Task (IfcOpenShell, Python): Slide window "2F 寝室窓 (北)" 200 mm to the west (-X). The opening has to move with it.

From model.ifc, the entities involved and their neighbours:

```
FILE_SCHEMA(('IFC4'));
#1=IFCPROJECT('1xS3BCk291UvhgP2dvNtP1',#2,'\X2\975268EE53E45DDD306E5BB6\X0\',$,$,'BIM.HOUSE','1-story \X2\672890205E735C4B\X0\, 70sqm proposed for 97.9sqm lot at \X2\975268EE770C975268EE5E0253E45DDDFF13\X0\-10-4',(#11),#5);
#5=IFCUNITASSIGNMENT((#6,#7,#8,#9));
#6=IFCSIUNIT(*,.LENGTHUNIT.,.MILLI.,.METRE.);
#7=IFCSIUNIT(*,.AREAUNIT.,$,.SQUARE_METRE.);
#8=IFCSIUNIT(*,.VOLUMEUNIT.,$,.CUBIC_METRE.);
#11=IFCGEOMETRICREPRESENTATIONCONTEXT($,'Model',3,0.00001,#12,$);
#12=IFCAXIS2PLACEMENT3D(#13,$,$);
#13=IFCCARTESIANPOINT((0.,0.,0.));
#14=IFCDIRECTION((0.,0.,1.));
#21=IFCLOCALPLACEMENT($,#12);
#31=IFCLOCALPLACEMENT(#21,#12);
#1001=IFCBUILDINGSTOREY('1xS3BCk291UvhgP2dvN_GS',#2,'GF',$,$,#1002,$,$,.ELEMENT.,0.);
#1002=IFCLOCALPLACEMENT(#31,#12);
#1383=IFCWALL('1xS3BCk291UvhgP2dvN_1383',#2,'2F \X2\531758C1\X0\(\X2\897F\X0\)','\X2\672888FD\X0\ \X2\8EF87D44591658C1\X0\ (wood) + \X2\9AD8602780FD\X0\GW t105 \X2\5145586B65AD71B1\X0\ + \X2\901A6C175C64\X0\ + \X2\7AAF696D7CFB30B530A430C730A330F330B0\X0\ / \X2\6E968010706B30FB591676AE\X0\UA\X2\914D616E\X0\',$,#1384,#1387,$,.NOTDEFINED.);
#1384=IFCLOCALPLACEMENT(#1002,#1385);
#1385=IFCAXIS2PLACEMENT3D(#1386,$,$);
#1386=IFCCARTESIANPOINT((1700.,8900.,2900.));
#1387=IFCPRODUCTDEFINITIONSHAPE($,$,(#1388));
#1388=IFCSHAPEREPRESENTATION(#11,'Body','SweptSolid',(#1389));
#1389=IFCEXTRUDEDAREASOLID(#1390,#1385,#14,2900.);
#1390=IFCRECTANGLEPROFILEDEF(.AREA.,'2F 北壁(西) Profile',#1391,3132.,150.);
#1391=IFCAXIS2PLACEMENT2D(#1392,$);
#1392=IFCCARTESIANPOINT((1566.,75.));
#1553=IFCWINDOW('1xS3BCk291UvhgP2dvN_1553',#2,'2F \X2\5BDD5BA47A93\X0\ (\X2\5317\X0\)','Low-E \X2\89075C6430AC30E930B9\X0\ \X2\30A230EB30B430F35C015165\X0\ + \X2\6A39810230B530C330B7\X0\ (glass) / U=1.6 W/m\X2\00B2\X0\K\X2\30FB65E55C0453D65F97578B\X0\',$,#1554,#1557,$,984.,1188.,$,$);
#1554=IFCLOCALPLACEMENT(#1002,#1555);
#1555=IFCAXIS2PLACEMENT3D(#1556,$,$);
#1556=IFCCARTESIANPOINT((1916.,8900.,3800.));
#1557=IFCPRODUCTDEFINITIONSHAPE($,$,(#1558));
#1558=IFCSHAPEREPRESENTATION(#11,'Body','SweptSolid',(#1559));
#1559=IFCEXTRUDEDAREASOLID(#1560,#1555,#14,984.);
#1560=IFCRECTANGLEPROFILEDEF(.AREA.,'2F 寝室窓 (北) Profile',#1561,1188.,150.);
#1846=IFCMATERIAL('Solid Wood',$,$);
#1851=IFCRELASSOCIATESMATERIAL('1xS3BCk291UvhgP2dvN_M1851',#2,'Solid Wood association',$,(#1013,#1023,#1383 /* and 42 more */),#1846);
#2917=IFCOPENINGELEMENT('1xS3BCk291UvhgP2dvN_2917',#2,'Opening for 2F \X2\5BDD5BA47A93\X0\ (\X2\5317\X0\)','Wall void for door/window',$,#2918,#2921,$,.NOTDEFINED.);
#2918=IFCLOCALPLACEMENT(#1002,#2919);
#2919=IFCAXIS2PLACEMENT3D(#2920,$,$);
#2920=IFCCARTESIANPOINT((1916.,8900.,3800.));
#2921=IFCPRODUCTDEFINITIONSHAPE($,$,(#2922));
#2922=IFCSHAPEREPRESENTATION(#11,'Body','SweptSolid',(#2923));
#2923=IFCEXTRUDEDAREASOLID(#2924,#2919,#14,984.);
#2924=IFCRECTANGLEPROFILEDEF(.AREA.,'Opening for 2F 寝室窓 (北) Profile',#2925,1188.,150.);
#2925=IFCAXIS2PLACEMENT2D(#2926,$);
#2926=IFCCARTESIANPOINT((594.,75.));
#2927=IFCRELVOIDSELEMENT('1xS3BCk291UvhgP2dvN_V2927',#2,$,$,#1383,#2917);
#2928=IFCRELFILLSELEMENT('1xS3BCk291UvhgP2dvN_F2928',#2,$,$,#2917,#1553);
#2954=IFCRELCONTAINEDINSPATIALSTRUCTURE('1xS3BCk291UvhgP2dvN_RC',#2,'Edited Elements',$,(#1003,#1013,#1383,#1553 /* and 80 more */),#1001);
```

```python
import ifcopenshell
import ifcopenshell.api.geometry
import ifcopenshell.util.placement

model = ifcopenshell.open("model.ifc")

window = model.by_guid("1xS3BCk291UvhgP2dvN_1553")
opening = window.FillsVoids[0].RelatingOpeningElement
wall = opening.VoidsElements[0].RelatingBuildingElement

wall_matrix = ifcopenshell.util.placement.get_local_placement(wall.ObjectPlacement)
shift = wall_matrix[:3, 0] * -200.0
before = ifcopenshell.util.placement.get_local_placement(window.ObjectPlacement)[:3, 3].copy()

# The window is not placed relative to its opening, so move both.
for product in (opening, window):
    matrix = ifcopenshell.util.placement.get_local_placement(product.ObjectPlacement)
    matrix[:3, 3] += shift
    ifcopenshell.api.geometry.edit_object_placement(model, product=product, matrix=matrix, is_si=False)

after = ifcopenshell.util.placement.get_local_placement(window.ObjectPlacement)[:3, 3]
print("window moved by", (after - before).round(3) + 0.0)

model.write("model_rev.ifc")
```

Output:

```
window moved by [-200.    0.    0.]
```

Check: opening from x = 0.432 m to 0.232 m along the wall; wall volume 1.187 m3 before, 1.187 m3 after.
